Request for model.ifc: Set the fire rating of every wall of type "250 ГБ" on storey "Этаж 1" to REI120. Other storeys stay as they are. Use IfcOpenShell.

First a look at what the model holds.

```python
import ifcopenshell
import ifcopenshell.util.element

model = ifcopenshell.open("model.ifc")
print(model.schema)
storey = next(s for s in model.by_type("IfcBuildingStorey") if s.Name == "Этаж 1")
walls = [e for e in ifcopenshell.util.element.get_decomposition(storey) if e.is_a("IfcWall")]
seen = {}
for e in walls:
    element_type = ifcopenshell.util.element.get_type(e)
    key = (element_type.Name if element_type != e and element_type else None, ifcopenshell.util.element.get_pset(e, "Pset_WallCommon", "FireRating"))
    seen[key] = seen.get(key, 0) + 1
for (name, value), count in sorted(seen.items(), key=str):
    print(count, "x", name, "|", value)
```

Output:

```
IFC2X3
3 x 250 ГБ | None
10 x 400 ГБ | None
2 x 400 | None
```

```python
import ifcopenshell
import ifcopenshell.api.pset
import ifcopenshell.util.element

model = ifcopenshell.open("model.ifc")

storey = next(s for s in model.by_type("IfcBuildingStorey") if s.Name == "Этаж 1")
walls = [e for e in ifcopenshell.util.element.get_decomposition(storey) if e.is_a("IfcWall")]

count = 0
for e in walls:
    element_type = ifcopenshell.util.element.get_type(e)
    if element_type in (None, e) or element_type.Name != "250 ГБ":
        continue
    # add_pset returns the element's existing set when there is one.
    pset = ifcopenshell.api.pset.add_pset(model, product=e, name="Pset_WallCommon")
    ifcopenshell.api.pset.edit_pset(model, pset=pset, properties={"FireRating": "REI120"})
    count += 1

print(count, "walls updated")

model.write("model_edited.ifc")
```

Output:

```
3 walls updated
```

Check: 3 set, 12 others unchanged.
